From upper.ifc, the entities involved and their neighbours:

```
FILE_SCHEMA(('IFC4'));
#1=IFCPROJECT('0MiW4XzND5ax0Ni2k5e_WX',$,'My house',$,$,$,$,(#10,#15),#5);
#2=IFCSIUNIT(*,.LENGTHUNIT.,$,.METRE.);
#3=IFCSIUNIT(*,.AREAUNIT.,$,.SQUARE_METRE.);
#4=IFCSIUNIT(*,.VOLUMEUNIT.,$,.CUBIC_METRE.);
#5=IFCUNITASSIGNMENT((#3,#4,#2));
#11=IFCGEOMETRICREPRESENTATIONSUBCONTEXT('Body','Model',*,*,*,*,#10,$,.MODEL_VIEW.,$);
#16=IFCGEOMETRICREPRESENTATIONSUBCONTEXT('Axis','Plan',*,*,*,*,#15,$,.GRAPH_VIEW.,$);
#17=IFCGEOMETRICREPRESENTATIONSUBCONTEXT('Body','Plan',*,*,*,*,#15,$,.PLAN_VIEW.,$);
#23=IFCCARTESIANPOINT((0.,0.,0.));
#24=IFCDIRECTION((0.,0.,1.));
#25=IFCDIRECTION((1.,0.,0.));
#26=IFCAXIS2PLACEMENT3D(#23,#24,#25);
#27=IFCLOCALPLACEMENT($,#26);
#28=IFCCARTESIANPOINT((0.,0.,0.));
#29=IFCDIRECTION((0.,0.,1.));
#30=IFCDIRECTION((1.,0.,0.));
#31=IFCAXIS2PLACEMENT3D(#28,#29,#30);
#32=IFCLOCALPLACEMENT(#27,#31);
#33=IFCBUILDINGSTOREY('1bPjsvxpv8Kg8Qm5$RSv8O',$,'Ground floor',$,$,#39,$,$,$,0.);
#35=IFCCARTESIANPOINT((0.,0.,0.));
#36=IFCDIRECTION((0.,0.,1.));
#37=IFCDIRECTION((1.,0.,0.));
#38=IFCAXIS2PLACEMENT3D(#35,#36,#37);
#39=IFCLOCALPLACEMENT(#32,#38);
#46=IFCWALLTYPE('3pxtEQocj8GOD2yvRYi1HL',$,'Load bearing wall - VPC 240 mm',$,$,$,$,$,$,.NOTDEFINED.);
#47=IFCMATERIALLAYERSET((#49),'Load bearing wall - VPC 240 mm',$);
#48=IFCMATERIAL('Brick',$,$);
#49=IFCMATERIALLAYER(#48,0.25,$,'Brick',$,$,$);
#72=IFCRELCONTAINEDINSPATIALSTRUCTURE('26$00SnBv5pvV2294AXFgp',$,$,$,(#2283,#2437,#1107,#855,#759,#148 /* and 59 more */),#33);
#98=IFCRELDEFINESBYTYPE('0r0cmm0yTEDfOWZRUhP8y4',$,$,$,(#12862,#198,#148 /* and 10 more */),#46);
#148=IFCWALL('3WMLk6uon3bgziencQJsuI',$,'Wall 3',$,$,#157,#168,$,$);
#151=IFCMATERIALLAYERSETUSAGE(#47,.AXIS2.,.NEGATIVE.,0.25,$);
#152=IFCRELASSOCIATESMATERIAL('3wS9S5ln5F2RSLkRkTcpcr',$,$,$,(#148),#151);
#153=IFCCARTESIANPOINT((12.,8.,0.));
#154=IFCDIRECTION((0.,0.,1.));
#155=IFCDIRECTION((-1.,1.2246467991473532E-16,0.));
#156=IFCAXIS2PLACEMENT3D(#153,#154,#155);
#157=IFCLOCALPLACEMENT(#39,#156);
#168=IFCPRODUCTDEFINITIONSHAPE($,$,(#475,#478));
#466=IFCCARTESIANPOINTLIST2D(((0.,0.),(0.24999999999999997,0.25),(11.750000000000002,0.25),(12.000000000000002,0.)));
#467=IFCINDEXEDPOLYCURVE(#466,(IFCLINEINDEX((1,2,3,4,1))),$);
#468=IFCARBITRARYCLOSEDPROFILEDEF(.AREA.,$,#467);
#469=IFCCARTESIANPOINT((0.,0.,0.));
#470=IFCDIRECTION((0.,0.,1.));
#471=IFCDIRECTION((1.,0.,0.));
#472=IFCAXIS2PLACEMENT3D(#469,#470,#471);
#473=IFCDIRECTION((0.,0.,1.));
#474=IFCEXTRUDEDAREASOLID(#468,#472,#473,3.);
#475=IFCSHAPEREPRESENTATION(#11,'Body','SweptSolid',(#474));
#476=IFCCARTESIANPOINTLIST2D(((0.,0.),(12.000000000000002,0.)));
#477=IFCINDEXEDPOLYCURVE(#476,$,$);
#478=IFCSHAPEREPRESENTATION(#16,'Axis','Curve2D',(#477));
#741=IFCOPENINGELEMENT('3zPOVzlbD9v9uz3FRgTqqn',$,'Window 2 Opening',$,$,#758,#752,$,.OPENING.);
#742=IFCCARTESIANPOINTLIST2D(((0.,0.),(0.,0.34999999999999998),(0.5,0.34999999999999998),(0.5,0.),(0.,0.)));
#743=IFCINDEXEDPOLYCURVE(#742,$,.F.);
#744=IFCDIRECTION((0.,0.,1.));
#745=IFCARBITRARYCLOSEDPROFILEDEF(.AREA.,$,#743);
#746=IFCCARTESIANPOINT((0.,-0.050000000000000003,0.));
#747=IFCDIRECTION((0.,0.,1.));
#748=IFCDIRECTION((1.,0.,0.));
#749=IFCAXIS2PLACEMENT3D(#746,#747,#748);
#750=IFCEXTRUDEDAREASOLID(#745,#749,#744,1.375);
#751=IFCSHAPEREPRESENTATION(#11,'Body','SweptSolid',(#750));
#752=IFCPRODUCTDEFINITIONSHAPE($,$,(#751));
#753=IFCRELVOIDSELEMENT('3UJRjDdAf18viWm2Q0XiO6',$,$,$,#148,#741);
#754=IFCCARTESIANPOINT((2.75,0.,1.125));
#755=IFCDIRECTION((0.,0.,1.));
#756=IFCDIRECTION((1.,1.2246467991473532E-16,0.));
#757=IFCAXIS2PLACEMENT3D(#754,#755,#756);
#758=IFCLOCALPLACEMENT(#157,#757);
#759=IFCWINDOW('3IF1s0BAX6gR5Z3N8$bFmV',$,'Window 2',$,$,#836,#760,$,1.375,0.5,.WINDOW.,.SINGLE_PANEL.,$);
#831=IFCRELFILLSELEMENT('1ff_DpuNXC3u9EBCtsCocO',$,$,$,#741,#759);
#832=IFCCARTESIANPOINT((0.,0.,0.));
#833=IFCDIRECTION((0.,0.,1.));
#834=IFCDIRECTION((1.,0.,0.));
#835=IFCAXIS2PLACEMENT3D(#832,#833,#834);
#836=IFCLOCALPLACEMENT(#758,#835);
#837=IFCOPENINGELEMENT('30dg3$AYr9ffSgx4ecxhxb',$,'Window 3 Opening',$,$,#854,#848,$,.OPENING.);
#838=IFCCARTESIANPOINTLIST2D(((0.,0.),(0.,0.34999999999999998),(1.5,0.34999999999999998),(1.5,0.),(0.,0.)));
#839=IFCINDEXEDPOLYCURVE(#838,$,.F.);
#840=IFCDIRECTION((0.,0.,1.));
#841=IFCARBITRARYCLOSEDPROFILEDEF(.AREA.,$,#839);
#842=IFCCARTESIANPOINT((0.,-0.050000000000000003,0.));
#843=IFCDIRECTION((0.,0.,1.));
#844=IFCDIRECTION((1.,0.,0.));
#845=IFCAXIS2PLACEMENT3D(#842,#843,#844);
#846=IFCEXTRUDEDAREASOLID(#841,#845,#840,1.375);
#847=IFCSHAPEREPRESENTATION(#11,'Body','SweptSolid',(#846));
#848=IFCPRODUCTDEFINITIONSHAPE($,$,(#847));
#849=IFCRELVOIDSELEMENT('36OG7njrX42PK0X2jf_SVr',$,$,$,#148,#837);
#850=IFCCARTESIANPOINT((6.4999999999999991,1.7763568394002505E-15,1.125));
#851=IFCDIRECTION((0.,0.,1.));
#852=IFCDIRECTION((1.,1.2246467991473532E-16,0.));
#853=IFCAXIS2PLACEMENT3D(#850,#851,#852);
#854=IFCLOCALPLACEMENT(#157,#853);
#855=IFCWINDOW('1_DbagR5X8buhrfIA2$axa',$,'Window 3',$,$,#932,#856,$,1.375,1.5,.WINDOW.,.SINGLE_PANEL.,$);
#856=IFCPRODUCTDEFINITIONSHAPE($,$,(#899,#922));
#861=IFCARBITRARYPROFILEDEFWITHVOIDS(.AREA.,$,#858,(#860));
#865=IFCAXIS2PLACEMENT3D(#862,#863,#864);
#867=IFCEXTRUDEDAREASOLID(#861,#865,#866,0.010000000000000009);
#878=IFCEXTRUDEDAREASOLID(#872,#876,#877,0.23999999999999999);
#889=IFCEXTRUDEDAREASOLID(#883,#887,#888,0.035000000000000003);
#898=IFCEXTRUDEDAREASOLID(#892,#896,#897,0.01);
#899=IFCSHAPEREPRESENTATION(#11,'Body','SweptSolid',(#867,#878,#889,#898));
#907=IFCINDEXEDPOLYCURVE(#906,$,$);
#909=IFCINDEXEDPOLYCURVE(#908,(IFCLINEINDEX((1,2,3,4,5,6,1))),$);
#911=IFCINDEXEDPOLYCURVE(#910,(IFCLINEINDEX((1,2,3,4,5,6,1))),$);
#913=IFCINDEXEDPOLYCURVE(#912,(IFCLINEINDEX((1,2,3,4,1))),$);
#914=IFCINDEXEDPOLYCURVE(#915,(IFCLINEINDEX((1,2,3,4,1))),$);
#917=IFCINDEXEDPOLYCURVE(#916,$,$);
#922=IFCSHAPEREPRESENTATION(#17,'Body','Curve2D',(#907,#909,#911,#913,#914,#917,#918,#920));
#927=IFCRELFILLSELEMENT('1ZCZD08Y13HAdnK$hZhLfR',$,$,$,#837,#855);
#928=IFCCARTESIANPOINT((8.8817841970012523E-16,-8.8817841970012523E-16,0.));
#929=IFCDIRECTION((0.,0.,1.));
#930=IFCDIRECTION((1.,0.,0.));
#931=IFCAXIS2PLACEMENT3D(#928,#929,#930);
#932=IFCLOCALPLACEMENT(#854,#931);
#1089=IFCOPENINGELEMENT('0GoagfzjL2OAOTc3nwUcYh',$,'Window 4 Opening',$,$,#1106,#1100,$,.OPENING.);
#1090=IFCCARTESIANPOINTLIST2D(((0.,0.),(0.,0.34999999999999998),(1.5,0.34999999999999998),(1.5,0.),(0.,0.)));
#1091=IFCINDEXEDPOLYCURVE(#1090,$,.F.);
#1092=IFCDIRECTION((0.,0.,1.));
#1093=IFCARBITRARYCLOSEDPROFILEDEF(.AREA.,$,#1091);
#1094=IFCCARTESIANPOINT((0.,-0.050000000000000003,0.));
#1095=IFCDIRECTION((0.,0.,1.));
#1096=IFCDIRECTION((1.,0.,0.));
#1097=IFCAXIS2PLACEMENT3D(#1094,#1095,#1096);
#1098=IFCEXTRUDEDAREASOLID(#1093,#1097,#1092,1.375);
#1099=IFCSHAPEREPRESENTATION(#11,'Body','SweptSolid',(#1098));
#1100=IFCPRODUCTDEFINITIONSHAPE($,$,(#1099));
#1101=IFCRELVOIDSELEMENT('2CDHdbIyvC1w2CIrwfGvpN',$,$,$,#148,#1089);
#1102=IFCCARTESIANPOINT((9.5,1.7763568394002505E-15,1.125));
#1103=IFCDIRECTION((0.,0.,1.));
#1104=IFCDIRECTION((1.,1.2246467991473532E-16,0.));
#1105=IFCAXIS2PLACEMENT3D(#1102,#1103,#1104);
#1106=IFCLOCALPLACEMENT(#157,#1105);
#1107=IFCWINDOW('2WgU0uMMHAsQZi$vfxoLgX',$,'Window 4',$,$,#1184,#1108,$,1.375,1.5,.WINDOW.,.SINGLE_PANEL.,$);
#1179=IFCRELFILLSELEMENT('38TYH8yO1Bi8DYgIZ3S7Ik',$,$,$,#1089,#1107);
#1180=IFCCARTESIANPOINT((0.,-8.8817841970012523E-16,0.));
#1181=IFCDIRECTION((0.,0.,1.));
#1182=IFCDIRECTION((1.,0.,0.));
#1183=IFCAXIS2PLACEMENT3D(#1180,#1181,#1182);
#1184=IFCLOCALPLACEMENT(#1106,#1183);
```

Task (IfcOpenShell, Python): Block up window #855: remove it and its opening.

```python
import ifcopenshell
import ifcopenshell.api.feature
import ifcopenshell.api.root
import ifcopenshell.geom
import ifcopenshell.util.shape

model = ifcopenshell.open("upper.ifc")
settings = ifcopenshell.geom.settings()


def volume(element):
    """Net volume in cubic metres, openings subtracted."""
    shape = ifcopenshell.geom.create_shape(settings, element)
    return ifcopenshell.util.shape.get_volume(shape.geometry)


window = model.by_guid("1_DbagR5X8buhrfIA2$axa")
opening = window.FillsVoids[0].RelatingOpeningElement
wall = opening.VoidsElements[0].RelatingBuildingElement
before = volume(wall)

ifcopenshell.api.root.remove_product(model, product=window)
ifcopenshell.api.feature.remove_feature(model, feature=opening)

after = volume(wall)

print(f"wall volume {before:.3f} -> {after:.3f} m3")

model.write("upper_v2.ifc")
```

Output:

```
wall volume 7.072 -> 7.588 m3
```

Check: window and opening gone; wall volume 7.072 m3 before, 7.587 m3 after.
